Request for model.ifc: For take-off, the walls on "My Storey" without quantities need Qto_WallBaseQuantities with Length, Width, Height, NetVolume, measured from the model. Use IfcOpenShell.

First a look at what the model holds.

```python
import ifcopenshell
import ifcopenshell.util.element
import ifcopenshell.util.unit

model = ifcopenshell.open("model.ifc")
print(model.schema)
for unit_type in ("LENGTHUNIT", "AREAUNIT", "VOLUMEUNIT"):
    print(unit_type, ifcopenshell.util.unit.calculate_unit_scale(model, unit_type))
storey = next(s for s in model.by_type("IfcBuildingStorey") if s.Name == "My Storey")
walls = [e for e in ifcopenshell.util.element.get_decomposition(storey) if e.is_a("IfcWall")]
for e in sorted(walls, key=lambda e: e.id()):
    print(e.id(), e.is_a(), e.Name, list(ifcopenshell.util.element.get_psets(e, qtos_only=True)), sep=" | ")
```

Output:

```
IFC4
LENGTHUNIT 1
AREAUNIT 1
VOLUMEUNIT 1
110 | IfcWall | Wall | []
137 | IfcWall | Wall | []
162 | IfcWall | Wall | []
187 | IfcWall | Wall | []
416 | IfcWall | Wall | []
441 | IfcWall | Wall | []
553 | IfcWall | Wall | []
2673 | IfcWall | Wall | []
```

```python
import ifcopenshell
import ifcopenshell.api.pset
import ifcopenshell.geom
import ifcopenshell.util.element
import ifcopenshell.util.shape
import ifcopenshell.util.unit

model = ifcopenshell.open("model.ifc")
unit_scale = ifcopenshell.util.unit.calculate_unit_scale(model)
volume_scale = ifcopenshell.util.unit.calculate_unit_scale(model, "VOLUMEUNIT")
settings = ifcopenshell.geom.settings()

storey = next(s for s in model.by_type("IfcBuildingStorey") if s.Name == "My Storey")
walls = [e for e in ifcopenshell.util.element.get_decomposition(storey) if e.is_a("IfcWall")]

for e in sorted(walls, key=lambda e: e.id()):
    if ifcopenshell.util.element.get_psets(e, qtos_only=True, should_inherit=False):
        continue
    # Geometry comes back in metres, in the element's own axes.
    shape = ifcopenshell.geom.create_shape(settings, e)
    values = {
        "Length": ifcopenshell.util.shape.get_x(shape.geometry) / unit_scale,
        "Width": ifcopenshell.util.shape.get_y(shape.geometry) / unit_scale,
        "Height": ifcopenshell.util.shape.get_z(shape.geometry) / unit_scale,
        "NetVolume": ifcopenshell.util.shape.get_volume(shape.geometry) / volume_scale,
    }
    qto = ifcopenshell.api.pset.add_qto(model, product=e, name="Qto_WallBaseQuantities")
    ifcopenshell.api.pset.edit_qto(model, qto=qto, properties=values)
    print(e.id(), {k: round(v, 3) for k, v in values.items()})

model.write("model-out.ifc")
```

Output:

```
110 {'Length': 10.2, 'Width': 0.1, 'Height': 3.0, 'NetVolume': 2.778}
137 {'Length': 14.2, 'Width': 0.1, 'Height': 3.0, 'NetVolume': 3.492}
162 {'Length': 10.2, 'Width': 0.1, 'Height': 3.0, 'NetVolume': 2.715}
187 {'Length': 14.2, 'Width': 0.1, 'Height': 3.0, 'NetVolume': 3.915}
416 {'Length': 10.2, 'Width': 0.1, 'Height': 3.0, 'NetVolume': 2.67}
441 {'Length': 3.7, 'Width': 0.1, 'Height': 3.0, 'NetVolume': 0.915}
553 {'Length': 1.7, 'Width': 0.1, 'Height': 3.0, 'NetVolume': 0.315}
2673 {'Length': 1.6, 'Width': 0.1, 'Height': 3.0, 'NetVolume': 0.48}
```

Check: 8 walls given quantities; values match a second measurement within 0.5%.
